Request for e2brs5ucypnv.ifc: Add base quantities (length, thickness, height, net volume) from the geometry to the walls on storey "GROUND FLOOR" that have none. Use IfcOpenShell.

First a look at what the model holds.

```python
import ifcopenshell
import ifcopenshell.util.element
import ifcopenshell.util.unit

model = ifcopenshell.open("e2brs5ucypnv.ifc")
print(model.schema)
for unit_type in ("LENGTHUNIT", "AREAUNIT", "VOLUMEUNIT"):
    print(unit_type, ifcopenshell.util.unit.calculate_unit_scale(model, unit_type))
storey = next(s for s in model.by_type("IfcBuildingStorey") if s.Name == "GROUND FLOOR")
walls = [e for e in ifcopenshell.util.element.get_decomposition(storey) if e.is_a("IfcWall")]
for e in sorted(walls, key=lambda e: e.id()):
    print(e.id(), e.is_a(), e.Name, list(ifcopenshell.util.element.get_psets(e, qtos_only=True)), sep=" | ")
```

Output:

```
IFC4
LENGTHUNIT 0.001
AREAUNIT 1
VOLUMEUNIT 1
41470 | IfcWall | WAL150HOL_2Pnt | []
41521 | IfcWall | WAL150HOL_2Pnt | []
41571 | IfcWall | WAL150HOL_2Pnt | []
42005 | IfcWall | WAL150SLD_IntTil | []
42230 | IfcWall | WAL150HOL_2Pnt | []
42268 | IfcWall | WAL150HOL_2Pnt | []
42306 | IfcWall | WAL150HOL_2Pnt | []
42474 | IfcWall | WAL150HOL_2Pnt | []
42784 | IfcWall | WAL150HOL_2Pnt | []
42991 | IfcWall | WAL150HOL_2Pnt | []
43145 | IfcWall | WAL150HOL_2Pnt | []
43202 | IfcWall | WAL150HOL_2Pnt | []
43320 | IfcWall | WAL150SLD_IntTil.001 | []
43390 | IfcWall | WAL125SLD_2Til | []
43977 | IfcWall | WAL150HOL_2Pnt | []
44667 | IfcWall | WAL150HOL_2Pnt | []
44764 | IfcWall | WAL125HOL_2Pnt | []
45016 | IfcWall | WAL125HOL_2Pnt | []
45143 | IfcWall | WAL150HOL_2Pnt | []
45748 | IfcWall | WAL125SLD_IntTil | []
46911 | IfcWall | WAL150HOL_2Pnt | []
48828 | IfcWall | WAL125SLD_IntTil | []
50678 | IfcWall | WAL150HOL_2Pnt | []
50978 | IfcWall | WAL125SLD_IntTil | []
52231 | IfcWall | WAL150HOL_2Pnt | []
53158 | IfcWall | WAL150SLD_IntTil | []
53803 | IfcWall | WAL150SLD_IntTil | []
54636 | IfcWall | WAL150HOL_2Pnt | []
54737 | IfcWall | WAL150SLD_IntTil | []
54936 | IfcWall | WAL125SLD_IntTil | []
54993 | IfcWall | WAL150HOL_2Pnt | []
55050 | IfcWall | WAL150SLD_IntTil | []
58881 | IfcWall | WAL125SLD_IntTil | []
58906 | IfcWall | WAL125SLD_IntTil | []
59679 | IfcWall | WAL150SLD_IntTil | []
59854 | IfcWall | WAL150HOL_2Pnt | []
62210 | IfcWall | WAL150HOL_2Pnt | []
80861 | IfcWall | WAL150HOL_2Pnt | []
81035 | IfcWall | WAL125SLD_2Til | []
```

```python
import ifcopenshell
import ifcopenshell.api.pset
import ifcopenshell.geom
import ifcopenshell.util.element
import ifcopenshell.util.shape
import ifcopenshell.util.unit

model = ifcopenshell.open("e2brs5ucypnv.ifc")
unit_scale = ifcopenshell.util.unit.calculate_unit_scale(model)
volume_scale = ifcopenshell.util.unit.calculate_unit_scale(model, "VOLUMEUNIT")
settings = ifcopenshell.geom.settings()

storey = next(s for s in model.by_type("IfcBuildingStorey") if s.Name == "GROUND FLOOR")
walls = [e for e in ifcopenshell.util.element.get_decomposition(storey) if e.is_a("IfcWall")]

for e in sorted(walls, key=lambda e: e.id()):
    if ifcopenshell.util.element.get_psets(e, qtos_only=True, should_inherit=False):
        continue
    # Geometry comes back in metres, in the element's own axes.
    shape = ifcopenshell.geom.create_shape(settings, e)
    values = {
        "Length": ifcopenshell.util.shape.get_x(shape.geometry) / unit_scale,
        "Width": ifcopenshell.util.shape.get_y(shape.geometry) / unit_scale,
        "Height": ifcopenshell.util.shape.get_z(shape.geometry) / unit_scale,
        "NetVolume": ifcopenshell.util.shape.get_volume(shape.geometry) / volume_scale,
    }
    qto = ifcopenshell.api.pset.add_qto(model, product=e, name="Qto_WallBaseQuantities")
    ifcopenshell.api.pset.edit_qto(model, qto=qto, properties=values)
    print(e.id(), {k: round(v, 3) for k, v in values.items()})

model.write("e2brs5ucypnv_edited.ifc")
```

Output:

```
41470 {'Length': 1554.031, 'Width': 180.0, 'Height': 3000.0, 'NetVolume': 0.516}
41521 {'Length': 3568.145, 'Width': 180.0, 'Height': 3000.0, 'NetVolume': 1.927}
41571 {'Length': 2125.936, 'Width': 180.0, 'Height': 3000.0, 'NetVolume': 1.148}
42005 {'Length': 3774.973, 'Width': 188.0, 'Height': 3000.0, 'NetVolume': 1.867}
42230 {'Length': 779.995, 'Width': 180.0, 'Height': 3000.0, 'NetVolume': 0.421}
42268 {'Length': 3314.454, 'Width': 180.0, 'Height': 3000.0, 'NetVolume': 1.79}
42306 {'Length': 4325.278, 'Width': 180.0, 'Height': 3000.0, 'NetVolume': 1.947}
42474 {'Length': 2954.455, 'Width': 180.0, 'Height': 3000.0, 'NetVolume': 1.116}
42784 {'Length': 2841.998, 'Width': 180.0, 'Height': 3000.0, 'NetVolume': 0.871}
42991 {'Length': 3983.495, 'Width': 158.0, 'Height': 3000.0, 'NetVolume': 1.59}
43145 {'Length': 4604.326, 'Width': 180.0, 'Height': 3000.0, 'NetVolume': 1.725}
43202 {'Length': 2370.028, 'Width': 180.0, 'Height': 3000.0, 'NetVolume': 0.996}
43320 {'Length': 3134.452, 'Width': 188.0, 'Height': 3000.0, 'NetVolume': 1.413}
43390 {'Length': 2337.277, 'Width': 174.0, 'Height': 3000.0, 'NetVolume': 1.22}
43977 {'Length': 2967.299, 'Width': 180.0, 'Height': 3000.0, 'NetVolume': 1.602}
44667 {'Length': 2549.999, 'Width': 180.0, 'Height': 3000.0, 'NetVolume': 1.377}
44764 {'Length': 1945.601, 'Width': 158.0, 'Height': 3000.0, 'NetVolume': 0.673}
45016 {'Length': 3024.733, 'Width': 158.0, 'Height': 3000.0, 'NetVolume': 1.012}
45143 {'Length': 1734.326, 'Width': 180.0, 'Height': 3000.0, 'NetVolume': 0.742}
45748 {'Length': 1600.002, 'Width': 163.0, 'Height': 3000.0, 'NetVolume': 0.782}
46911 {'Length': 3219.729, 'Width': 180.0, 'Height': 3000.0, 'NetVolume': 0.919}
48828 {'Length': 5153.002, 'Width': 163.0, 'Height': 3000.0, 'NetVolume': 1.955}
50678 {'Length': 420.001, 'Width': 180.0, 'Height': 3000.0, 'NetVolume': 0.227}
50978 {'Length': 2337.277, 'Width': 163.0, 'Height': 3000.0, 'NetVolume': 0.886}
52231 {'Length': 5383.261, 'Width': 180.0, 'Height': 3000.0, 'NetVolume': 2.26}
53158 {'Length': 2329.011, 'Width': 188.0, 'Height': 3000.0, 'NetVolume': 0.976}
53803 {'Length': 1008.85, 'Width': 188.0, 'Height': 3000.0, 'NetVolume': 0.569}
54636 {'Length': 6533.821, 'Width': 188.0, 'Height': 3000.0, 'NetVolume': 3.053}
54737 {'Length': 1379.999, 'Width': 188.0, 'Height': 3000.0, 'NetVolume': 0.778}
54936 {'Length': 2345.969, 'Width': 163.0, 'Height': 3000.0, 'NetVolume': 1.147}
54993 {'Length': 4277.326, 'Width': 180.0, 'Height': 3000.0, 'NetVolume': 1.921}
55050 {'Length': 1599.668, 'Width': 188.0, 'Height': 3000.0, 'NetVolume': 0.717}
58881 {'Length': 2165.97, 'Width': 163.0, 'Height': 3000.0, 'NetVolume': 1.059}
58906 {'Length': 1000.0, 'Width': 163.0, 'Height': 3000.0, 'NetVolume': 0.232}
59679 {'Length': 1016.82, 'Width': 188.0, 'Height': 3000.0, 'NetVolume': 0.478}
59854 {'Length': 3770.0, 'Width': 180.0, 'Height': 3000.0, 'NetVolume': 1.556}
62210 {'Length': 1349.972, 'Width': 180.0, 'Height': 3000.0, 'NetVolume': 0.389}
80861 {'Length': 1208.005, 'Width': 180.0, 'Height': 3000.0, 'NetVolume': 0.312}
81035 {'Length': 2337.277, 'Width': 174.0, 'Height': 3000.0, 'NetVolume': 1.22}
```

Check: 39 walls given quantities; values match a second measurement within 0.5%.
